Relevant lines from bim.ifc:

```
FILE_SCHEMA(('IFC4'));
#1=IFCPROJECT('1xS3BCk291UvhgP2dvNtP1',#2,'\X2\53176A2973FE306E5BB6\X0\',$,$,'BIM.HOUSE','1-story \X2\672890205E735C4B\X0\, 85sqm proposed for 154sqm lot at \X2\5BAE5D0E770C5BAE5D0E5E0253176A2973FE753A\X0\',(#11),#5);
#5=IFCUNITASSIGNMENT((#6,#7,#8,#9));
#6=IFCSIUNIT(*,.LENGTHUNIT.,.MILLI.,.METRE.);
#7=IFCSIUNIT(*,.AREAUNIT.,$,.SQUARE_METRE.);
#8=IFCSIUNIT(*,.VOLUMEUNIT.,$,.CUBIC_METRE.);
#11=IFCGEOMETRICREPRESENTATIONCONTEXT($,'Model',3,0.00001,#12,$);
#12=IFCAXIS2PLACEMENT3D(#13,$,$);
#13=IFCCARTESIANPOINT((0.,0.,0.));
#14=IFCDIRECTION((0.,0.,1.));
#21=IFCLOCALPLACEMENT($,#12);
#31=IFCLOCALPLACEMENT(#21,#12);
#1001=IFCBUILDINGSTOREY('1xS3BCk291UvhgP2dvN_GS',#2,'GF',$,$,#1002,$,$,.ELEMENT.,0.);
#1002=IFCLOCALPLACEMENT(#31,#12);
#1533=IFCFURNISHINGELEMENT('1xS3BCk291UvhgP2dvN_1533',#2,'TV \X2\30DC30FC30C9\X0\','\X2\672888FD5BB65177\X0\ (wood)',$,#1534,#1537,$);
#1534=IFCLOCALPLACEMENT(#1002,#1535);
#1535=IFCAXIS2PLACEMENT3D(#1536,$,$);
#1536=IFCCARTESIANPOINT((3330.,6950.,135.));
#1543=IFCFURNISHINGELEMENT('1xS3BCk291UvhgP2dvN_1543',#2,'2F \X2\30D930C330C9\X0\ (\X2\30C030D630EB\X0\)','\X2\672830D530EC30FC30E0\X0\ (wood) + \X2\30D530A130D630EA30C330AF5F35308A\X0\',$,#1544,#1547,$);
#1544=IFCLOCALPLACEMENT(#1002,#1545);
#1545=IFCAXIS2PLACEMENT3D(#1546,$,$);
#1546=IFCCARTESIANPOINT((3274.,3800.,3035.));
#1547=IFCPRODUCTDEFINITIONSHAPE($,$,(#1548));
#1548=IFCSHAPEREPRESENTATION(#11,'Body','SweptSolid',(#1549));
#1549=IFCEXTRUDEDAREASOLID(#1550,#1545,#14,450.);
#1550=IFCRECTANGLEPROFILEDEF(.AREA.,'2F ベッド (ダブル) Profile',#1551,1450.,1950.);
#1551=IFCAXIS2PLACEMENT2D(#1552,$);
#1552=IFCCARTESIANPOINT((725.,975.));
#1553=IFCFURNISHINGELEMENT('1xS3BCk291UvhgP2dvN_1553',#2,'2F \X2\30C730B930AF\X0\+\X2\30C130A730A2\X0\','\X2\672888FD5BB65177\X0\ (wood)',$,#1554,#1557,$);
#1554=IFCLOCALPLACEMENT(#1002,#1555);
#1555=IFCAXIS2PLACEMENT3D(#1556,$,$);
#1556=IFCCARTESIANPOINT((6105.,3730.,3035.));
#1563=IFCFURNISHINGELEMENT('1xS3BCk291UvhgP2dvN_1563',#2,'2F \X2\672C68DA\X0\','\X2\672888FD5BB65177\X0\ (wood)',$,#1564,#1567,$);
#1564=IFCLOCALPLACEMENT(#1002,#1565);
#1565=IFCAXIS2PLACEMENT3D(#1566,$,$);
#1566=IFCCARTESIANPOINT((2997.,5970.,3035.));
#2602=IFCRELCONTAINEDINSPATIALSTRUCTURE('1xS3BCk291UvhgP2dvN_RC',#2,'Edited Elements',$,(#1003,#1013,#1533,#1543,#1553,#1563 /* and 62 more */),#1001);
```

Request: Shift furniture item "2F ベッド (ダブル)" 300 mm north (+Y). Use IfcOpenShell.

```python
import ifcopenshell
import ifcopenshell.api.geometry
import ifcopenshell.util.placement
import ifcopenshell.util.unit

model = ifcopenshell.open("bim.ifc")
unit_scale = ifcopenshell.util.unit.calculate_unit_scale(model)

item = model.by_guid("1xS3BCk291UvhgP2dvN_1543")
matrix = ifcopenshell.util.placement.get_local_placement(item.ObjectPlacement)
matrix[1, 3] += 0.3 / unit_scale
ifcopenshell.api.geometry.edit_object_placement(model, product=item, matrix=matrix, is_si=False)

print(ifcopenshell.util.placement.get_local_placement(item.ObjectPlacement).round(3) + 0.0)

model.write("bim_updated.ifc")
```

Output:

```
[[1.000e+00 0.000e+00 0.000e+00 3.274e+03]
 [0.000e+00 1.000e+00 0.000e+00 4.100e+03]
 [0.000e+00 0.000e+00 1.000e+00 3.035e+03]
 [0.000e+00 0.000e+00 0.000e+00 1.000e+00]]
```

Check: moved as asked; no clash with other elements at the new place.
